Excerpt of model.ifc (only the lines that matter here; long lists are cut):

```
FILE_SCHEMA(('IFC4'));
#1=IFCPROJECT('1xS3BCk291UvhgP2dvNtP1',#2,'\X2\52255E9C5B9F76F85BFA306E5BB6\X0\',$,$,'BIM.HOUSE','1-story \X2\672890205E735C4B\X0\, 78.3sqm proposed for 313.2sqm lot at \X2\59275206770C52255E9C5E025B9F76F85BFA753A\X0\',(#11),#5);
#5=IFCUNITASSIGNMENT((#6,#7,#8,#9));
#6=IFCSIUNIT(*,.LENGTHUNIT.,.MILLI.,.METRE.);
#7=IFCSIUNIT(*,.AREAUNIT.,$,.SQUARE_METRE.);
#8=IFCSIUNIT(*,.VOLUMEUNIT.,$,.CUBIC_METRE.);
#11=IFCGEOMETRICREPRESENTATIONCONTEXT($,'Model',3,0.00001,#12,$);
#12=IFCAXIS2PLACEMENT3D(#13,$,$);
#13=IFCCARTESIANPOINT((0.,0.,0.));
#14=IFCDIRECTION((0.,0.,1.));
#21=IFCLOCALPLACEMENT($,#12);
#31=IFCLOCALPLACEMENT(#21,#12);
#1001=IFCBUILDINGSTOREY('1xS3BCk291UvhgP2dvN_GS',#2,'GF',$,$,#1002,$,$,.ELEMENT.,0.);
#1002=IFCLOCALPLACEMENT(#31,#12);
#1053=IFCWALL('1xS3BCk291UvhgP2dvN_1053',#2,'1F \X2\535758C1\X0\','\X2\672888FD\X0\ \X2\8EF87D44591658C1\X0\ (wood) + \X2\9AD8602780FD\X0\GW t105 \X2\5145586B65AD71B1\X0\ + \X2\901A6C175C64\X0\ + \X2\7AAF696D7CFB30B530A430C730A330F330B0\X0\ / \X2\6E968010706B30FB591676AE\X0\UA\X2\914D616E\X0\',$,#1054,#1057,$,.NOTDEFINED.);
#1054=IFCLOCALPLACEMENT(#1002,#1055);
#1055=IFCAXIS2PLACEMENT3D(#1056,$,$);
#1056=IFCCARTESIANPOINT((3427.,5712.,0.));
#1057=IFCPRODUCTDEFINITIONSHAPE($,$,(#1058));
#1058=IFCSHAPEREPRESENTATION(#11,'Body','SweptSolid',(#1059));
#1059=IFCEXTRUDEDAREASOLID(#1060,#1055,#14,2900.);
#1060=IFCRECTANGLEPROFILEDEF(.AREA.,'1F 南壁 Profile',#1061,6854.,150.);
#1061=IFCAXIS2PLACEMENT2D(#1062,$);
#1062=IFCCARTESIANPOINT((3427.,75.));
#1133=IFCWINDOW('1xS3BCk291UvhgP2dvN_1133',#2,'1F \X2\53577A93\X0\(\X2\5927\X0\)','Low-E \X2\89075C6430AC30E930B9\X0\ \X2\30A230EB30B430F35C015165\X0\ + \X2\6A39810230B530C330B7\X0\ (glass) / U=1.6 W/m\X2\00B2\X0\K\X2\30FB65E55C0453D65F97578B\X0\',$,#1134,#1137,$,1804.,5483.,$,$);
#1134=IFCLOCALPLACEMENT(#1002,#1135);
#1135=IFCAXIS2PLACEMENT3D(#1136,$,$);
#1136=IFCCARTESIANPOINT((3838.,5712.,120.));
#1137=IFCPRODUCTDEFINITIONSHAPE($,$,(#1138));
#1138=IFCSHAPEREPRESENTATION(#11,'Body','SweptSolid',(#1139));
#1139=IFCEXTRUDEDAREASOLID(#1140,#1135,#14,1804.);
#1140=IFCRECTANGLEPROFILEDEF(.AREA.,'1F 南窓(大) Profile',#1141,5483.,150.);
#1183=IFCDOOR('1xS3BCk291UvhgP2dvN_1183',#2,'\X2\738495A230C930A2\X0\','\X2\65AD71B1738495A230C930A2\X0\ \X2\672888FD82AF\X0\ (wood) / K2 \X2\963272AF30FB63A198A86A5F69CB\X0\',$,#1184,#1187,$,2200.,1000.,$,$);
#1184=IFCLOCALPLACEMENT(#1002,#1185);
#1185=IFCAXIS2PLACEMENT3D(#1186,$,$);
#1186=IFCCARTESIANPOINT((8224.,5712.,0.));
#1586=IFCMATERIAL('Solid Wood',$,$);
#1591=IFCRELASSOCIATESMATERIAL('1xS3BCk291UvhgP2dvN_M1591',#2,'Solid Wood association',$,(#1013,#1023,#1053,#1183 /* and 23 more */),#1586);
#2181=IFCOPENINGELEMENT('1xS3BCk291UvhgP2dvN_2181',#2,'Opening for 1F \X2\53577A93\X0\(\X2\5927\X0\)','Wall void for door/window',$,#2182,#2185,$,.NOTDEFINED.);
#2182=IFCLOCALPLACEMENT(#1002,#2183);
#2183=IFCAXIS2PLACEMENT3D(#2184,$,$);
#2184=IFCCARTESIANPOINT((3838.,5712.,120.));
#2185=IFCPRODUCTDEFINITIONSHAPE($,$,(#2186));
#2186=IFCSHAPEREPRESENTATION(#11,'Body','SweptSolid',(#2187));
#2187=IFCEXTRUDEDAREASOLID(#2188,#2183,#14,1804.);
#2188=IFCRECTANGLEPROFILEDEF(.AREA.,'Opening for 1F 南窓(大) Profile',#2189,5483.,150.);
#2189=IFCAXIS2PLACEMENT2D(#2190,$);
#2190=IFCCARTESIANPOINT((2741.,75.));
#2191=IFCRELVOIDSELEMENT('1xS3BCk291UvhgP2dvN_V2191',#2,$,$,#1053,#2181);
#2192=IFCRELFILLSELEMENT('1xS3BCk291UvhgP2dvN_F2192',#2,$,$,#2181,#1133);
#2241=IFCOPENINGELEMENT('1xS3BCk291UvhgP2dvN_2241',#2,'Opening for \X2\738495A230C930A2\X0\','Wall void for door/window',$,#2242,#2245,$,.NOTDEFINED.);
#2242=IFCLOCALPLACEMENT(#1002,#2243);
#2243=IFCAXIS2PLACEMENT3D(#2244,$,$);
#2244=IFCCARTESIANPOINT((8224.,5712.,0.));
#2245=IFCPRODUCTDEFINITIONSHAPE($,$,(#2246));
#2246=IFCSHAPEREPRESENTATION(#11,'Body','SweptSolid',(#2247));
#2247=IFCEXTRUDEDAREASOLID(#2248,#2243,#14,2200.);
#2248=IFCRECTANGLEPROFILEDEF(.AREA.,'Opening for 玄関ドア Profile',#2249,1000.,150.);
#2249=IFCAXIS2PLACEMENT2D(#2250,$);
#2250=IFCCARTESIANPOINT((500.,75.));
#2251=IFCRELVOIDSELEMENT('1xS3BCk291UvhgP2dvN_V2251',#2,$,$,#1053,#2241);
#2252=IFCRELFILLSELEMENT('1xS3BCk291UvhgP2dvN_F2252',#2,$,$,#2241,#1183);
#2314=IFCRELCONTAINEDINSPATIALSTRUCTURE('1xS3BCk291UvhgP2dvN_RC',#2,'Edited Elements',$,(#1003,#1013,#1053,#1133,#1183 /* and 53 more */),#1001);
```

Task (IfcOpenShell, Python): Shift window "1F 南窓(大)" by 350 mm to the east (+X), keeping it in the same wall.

```python
import ifcopenshell
import ifcopenshell.api.geometry
import ifcopenshell.util.placement

model = ifcopenshell.open("model.ifc")

window = model.by_id(1133)
opening = window.FillsVoids[0].RelatingOpeningElement
wall = opening.VoidsElements[0].RelatingBuildingElement

wall_matrix = ifcopenshell.util.placement.get_local_placement(wall.ObjectPlacement)
shift = wall_matrix[:3, 0] * 350.0
before = ifcopenshell.util.placement.get_local_placement(window.ObjectPlacement)[:3, 3].copy()

# The window is not placed relative to its opening, so move both.
for product in (opening, window):
    matrix = ifcopenshell.util.placement.get_local_placement(product.ObjectPlacement)
    matrix[:3, 3] += shift
    ifcopenshell.api.geometry.edit_object_placement(model, product=product, matrix=matrix, is_si=False)

after = ifcopenshell.util.placement.get_local_placement(window.ObjectPlacement)[:3, 3]
print("window moved by", (after - before).round(3) + 0.0)

model.write("model_rev.ifc")
```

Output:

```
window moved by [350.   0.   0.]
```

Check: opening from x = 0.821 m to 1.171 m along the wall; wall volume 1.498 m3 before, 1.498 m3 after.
